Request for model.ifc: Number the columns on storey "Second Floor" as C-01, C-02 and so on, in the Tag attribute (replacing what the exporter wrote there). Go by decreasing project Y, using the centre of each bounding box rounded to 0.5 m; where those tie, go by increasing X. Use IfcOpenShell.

First a look at what the model holds.

```python
import ifcopenshell
import ifcopenshell.util.element
import ifcopenshell.util.placement

model = ifcopenshell.open("model.ifc")
print(model.schema)
storey = next(s for s in model.by_type("IfcBuildingStorey") if s.Name == "Second Floor")
columns = [e for e in ifcopenshell.util.element.get_decomposition(storey) if e.is_a("IfcColumn")]
for e in sorted(columns, key=lambda e: e.id()):
    origin = ifcopenshell.util.placement.get_local_placement(e.ObjectPlacement)[:3, 3]
    print(e.id(), e.Tag, e.Name, origin.round(2) + 0.0, sep=" | ")
```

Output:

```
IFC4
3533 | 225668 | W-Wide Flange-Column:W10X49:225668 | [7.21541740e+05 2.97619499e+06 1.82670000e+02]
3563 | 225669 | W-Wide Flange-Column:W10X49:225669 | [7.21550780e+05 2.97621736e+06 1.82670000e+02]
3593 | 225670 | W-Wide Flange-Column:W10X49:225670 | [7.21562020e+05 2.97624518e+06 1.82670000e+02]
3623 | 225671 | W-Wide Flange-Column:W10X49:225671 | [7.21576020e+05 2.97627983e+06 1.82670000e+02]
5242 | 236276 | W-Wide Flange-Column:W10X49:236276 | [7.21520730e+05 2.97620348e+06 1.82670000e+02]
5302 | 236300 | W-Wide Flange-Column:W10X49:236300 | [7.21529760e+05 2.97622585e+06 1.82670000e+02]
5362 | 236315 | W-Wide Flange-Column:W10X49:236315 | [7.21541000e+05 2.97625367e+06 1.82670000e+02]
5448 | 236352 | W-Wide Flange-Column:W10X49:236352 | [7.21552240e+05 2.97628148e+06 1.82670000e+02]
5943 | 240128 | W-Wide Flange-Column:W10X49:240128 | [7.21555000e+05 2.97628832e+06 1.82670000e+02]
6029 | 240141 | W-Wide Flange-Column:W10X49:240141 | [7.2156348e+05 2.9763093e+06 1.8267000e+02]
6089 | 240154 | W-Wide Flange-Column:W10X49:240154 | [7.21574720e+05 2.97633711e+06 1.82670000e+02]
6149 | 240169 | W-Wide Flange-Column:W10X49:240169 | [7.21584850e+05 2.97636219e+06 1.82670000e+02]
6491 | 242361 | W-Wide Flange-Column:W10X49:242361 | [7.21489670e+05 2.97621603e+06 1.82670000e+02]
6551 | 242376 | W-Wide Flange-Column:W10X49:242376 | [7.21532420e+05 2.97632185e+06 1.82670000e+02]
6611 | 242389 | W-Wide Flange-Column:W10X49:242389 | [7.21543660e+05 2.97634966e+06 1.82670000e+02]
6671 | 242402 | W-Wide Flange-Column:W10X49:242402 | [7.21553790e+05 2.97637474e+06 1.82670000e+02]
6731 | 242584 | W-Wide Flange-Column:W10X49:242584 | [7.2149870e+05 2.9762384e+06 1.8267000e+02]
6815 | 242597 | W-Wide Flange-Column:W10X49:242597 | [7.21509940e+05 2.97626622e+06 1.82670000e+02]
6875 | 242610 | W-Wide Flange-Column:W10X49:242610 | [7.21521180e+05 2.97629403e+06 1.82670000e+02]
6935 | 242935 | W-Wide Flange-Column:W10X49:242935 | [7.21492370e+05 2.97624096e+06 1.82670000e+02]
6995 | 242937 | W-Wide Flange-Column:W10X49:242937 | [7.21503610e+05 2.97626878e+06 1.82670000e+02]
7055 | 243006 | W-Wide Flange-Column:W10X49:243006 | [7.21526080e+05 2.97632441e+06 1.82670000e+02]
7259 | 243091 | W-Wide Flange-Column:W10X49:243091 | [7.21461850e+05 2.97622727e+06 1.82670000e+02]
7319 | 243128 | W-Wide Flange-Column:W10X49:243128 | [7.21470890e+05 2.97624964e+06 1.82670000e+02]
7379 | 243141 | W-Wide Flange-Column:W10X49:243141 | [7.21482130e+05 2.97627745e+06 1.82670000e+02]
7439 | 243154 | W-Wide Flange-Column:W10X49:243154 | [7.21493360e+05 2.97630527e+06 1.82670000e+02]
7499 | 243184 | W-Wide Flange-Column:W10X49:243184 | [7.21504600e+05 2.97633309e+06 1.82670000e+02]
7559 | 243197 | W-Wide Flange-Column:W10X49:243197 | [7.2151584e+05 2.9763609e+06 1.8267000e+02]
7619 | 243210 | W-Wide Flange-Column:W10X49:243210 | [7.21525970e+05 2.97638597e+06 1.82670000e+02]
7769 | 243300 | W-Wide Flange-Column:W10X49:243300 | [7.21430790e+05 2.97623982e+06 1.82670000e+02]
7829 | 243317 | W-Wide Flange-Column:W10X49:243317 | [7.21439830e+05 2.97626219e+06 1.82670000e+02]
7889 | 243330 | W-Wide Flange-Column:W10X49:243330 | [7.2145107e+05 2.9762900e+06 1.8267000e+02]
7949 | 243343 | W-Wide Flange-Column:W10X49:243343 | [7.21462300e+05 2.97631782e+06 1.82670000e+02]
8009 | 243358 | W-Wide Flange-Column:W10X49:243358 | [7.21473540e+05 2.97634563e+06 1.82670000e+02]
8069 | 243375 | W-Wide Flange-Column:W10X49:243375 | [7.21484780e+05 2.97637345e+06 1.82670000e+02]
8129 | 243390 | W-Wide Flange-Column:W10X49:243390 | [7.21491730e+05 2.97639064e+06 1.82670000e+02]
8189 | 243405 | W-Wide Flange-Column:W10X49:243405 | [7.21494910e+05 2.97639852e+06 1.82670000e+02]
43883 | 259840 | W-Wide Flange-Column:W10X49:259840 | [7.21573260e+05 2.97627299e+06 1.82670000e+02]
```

```python
import ifcopenshell
import ifcopenshell.geom
import ifcopenshell.util.element
import ifcopenshell.util.shape

model = ifcopenshell.open("model.ifc")
settings = ifcopenshell.geom.settings()
settings.set("use-world-coords", True)


def centre(element):
    shape = ifcopenshell.geom.create_shape(settings, element)
    return ifcopenshell.util.shape.get_bbox_centroid(shape.geometry)


storey = next(s for s in model.by_type("IfcBuildingStorey") if s.Name == "Second Floor")
columns = [e for e in ifcopenshell.util.element.get_decomposition(storey) if e.is_a("IfcColumn")]

# Insertion points can sit at a corner or the storey origin, so sort by the geometry (in metres).
centres = {e: centre(e) for e in columns}
columns.sort(key=lambda e: (-round(centres[e][1] / 0.5), centres[e][0]))

for i, e in enumerate(columns, start=1):
    number = f"C-{i:02d}"
    e.Tag = number
    print(e.id(), number)

model.write("model-out.ifc")
```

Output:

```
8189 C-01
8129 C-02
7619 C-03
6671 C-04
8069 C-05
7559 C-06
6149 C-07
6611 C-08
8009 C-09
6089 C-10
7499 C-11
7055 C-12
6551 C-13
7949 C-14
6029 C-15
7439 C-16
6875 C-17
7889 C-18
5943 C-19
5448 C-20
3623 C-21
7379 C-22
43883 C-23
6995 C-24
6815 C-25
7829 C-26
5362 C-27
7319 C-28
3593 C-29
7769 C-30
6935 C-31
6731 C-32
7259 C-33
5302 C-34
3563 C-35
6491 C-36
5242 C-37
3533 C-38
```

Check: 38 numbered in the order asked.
